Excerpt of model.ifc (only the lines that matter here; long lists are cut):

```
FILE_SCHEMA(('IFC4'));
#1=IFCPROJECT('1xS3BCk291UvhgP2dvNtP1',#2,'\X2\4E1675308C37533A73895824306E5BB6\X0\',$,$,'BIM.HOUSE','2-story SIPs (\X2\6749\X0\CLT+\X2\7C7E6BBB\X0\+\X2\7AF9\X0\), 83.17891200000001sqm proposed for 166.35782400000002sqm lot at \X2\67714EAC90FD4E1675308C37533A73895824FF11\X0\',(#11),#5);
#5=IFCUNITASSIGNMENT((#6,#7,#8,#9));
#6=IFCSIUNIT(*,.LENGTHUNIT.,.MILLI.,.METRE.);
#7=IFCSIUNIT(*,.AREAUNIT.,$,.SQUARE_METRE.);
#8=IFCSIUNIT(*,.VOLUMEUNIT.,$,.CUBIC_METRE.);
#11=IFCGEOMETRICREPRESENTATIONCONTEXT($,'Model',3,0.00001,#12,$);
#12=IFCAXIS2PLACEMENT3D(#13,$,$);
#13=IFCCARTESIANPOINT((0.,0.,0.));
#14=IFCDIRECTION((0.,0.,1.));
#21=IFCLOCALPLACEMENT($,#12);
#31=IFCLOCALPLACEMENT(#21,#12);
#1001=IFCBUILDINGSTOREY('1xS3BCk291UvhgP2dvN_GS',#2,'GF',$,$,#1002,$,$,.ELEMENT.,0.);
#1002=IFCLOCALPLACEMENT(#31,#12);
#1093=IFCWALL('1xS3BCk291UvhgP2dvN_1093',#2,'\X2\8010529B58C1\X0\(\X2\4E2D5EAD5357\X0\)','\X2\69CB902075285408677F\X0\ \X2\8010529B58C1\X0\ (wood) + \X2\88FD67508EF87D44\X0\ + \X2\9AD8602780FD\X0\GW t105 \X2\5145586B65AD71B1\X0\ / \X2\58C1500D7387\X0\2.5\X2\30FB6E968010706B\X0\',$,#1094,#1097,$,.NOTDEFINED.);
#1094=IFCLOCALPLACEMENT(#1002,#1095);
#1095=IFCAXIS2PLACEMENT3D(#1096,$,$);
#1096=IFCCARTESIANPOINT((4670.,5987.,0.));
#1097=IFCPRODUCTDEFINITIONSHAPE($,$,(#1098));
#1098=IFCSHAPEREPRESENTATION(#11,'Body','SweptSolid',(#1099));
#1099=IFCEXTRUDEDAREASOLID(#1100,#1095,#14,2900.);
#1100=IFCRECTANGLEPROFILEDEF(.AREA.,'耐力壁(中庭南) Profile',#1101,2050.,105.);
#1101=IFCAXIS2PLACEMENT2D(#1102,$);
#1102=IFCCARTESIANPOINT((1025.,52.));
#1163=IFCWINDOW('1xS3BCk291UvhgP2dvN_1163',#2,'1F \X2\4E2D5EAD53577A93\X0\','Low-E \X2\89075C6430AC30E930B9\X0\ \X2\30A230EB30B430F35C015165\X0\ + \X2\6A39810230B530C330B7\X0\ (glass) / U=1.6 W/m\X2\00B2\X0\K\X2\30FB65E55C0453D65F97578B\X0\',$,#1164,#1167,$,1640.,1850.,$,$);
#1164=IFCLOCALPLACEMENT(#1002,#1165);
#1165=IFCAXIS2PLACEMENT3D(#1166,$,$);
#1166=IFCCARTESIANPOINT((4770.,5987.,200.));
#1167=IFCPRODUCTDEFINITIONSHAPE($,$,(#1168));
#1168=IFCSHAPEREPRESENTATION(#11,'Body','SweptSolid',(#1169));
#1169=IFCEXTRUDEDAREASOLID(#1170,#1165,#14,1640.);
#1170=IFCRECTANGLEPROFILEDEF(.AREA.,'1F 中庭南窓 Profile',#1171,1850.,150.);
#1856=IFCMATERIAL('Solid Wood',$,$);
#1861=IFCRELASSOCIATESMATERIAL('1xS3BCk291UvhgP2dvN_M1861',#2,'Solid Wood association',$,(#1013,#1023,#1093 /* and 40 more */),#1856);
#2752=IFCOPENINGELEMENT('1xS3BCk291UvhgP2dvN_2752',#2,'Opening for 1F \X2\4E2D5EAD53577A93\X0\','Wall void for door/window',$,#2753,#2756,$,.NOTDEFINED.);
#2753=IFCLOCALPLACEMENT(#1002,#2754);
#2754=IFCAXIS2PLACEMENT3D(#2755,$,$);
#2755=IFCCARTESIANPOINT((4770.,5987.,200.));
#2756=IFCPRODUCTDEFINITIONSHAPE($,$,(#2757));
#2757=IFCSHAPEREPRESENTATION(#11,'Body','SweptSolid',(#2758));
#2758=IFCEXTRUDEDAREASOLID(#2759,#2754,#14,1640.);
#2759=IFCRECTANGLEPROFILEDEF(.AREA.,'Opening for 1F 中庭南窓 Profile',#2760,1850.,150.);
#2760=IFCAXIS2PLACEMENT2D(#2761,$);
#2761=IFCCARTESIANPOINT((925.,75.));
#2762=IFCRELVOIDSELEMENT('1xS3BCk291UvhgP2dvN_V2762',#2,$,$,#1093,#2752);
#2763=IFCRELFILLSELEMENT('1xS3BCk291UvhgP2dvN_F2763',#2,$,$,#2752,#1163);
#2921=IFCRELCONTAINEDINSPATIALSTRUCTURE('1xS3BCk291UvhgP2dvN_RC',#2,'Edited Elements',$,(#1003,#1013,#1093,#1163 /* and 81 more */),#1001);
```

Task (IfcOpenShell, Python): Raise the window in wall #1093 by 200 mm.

```python
import numpy as np
import ifcopenshell
import ifcopenshell.api.geometry
import ifcopenshell.util.placement
import ifcopenshell.util.unit

model = ifcopenshell.open("model.ifc")
unit_scale = ifcopenshell.util.unit.calculate_unit_scale(model)

window = model.by_guid("1xS3BCk291UvhgP2dvN_1163")
opening = window.FillsVoids[0].RelatingOpeningElement
dz = 0.2 / unit_scale

shift = np.array([0.0, 0.0, dz])
# The window is not placed relative to its opening, so move both.
for product in (opening, window):
    matrix = ifcopenshell.util.placement.get_local_placement(product.ObjectPlacement)
    matrix[:3, 3] += shift
    ifcopenshell.api.geometry.edit_object_placement(model, product=product, matrix=matrix, is_si=False)

print(f"moved by {dz * unit_scale:+.3f} m")

model.write("model_edited.ifc")
```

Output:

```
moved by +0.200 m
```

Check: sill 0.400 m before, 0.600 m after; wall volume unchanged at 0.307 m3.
